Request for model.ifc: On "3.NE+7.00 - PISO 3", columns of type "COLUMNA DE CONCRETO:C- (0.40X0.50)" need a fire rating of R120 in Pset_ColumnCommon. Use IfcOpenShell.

First a look at what the model holds.

```python
import ifcopenshell
import ifcopenshell.util.element

model = ifcopenshell.open("model.ifc")
print(model.schema)
storey = next(s for s in model.by_type("IfcBuildingStorey") if s.Name == "3.NE+7.00 - PISO 3")
columns = [e for e in ifcopenshell.util.element.get_decomposition(storey) if e.is_a("IfcColumn")]
seen = {}
for e in columns:
    element_type = ifcopenshell.util.element.get_type(e)
    key = (element_type.Name if element_type != e and element_type else None, ifcopenshell.util.element.get_pset(e, "Pset_ColumnCommon", "FireRating"))
    seen[key] = seen.get(key, 0) + 1
for (name, value), count in sorted(seen.items(), key=str):
    print(count, "x", name, "|", value)
```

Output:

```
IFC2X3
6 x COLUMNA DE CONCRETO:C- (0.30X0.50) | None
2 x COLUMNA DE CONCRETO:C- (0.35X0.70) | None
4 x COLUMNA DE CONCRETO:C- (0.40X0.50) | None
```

```python
import ifcopenshell
import ifcopenshell.api.pset
import ifcopenshell.util.element

model = ifcopenshell.open("model.ifc")

storey = next(s for s in model.by_type("IfcBuildingStorey") if s.Name == "3.NE+7.00 - PISO 3")
columns = [e for e in ifcopenshell.util.element.get_decomposition(storey) if e.is_a("IfcColumn")]

count = 0
for e in columns:
    element_type = ifcopenshell.util.element.get_type(e)
    if element_type in (None, e) or element_type.Name != "COLUMNA DE CONCRETO:C- (0.40X0.50)":
        continue
    # add_pset returns the element's existing set when there is one.
    pset = ifcopenshell.api.pset.add_pset(model, product=e, name="Pset_ColumnCommon")
    ifcopenshell.api.pset.edit_pset(model, pset=pset, properties={"FireRating": "R120"})
    count += 1

print(count, "columns updated")

model.write("model_rev.ifc")
```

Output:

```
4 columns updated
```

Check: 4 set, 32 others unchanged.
